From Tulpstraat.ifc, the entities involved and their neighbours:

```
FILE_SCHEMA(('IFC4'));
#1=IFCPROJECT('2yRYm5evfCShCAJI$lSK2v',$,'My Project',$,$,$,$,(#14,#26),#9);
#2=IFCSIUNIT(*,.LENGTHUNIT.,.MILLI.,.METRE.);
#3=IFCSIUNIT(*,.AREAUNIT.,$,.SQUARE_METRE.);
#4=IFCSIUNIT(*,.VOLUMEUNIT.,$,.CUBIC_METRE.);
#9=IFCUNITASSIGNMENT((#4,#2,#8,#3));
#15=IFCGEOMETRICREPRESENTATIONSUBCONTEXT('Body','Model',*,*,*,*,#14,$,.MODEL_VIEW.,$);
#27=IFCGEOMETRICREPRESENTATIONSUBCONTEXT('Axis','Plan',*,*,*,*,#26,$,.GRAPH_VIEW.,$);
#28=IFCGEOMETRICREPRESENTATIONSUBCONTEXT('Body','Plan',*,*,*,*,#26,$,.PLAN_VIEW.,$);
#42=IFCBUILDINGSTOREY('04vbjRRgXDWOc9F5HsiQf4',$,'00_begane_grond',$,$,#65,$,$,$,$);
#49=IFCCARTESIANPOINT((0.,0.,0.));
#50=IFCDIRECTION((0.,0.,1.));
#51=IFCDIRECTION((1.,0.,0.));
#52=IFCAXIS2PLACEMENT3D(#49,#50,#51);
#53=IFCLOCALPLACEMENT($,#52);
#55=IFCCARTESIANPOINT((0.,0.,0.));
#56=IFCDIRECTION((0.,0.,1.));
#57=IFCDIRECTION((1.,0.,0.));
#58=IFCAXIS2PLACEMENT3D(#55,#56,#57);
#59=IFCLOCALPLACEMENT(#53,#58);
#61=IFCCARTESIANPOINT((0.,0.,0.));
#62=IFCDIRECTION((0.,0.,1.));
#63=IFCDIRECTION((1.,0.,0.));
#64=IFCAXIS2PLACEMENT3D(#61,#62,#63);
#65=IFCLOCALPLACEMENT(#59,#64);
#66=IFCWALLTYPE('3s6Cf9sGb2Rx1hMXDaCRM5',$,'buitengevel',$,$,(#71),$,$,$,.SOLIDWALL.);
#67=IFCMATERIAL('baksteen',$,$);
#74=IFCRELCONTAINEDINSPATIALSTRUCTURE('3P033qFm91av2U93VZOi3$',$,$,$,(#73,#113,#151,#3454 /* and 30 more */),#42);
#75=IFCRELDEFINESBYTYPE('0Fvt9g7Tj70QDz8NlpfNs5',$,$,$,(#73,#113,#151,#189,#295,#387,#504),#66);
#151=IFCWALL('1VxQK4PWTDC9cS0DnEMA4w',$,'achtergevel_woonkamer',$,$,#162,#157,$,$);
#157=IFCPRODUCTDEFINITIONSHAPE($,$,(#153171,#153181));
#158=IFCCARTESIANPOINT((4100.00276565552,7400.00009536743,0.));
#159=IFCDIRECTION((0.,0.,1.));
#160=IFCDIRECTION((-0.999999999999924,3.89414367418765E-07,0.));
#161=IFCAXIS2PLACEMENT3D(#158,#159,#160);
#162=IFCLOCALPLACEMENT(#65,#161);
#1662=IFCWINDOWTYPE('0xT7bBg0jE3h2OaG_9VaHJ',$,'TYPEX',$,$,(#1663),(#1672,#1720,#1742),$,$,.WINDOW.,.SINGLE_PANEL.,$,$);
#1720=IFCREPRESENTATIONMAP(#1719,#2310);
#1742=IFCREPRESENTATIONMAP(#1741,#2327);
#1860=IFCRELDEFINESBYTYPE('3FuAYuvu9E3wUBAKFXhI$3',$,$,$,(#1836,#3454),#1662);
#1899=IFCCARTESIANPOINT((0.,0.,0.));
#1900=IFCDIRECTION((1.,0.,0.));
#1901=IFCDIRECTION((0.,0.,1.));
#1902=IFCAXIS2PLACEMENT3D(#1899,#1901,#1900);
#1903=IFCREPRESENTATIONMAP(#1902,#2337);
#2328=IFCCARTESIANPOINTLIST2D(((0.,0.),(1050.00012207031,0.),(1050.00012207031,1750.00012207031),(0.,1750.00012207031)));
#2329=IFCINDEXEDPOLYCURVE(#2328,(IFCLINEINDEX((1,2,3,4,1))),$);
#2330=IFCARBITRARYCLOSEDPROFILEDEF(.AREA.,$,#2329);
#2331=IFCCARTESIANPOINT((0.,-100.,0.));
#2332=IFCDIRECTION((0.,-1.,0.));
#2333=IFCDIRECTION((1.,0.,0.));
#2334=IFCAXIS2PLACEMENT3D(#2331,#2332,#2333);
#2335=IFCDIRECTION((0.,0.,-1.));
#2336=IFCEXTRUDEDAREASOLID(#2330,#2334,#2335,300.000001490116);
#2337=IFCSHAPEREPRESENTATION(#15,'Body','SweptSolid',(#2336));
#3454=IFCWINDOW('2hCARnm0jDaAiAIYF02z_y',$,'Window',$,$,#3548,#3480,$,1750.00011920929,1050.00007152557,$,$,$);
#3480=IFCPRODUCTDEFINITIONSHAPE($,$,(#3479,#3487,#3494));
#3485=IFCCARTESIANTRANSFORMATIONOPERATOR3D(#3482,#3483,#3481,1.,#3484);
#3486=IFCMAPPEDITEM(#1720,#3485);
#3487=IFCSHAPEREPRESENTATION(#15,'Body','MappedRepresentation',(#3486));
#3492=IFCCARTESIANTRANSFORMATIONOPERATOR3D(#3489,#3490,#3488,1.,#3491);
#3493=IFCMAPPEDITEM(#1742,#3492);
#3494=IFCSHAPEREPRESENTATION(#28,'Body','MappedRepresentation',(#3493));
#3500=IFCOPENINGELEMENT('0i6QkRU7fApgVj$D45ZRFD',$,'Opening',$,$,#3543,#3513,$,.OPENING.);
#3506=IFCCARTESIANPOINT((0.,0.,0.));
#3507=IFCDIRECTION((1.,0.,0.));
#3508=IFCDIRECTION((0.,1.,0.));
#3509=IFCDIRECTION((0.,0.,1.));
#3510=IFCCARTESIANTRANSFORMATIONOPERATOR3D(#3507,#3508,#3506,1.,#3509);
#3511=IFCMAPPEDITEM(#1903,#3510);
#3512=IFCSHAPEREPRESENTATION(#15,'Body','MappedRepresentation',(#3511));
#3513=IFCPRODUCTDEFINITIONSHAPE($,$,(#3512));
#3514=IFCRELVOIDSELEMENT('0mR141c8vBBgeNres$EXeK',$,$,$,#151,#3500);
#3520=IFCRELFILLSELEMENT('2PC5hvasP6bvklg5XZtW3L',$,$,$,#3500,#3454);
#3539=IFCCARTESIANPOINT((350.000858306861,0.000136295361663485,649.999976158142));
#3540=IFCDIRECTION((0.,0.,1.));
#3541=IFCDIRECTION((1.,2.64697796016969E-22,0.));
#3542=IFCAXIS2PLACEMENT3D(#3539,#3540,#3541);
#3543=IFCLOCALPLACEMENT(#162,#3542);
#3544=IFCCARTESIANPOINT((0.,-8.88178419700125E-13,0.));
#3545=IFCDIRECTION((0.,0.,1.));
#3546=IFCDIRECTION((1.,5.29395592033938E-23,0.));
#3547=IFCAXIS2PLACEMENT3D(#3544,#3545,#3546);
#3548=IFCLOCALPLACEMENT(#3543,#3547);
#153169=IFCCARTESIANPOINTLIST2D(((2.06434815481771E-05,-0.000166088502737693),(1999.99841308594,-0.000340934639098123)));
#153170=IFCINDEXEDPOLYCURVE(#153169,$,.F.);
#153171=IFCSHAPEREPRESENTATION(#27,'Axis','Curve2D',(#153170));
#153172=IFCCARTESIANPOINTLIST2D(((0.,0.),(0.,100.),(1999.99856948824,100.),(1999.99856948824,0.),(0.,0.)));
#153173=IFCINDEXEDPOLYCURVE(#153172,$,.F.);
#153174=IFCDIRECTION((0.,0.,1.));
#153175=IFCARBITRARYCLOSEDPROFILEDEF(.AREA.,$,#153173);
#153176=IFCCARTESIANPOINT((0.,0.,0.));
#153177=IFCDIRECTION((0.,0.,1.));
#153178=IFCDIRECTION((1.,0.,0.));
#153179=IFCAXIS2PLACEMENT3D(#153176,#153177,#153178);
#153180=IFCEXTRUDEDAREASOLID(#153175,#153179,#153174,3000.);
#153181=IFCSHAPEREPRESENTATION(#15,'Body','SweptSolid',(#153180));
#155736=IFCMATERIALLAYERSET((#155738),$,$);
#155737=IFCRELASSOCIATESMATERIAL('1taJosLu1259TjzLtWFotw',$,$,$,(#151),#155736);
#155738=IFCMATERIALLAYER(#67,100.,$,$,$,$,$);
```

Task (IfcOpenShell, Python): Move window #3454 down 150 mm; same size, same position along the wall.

```python
import numpy as np
import ifcopenshell
import ifcopenshell.api.geometry
import ifcopenshell.util.placement
import ifcopenshell.util.unit

model = ifcopenshell.open("Tulpstraat.ifc")
unit_scale = ifcopenshell.util.unit.calculate_unit_scale(model)

window = model.by_guid("2hCARnm0jDaAiAIYF02z_y")
opening = window.FillsVoids[0].RelatingOpeningElement
dz = -0.15 / unit_scale

shift = np.array([0.0, 0.0, dz])
# The window is placed relative to its opening, so it follows when the opening moves.
matrix = ifcopenshell.util.placement.get_local_placement(opening.ObjectPlacement)
matrix[:3, 3] += shift
ifcopenshell.api.geometry.edit_object_placement(
    model, product=opening, matrix=matrix, is_si=False, should_transform_children=True
)

print(f"moved by {dz * unit_scale:+.3f} m")

model.write("Tulpstraat_rev.ifc")
```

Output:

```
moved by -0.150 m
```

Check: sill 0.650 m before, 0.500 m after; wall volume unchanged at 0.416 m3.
